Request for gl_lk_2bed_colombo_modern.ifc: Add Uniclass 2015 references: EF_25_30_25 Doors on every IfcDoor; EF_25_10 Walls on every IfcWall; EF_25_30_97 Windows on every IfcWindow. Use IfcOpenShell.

First a look at what the model holds.

```python
import ifcopenshell

model = ifcopenshell.open("gl_lk_2bed_colombo_modern.ifc")
print(model.schema)
print("classifications:", [c.Name for c in model.by_type("IfcClassification")])
for ifc_class in ("IfcDoor", "IfcRoof", "IfcStair", "IfcWall", "IfcWindow"):
    print(ifc_class, len(model.by_type(ifc_class)))
```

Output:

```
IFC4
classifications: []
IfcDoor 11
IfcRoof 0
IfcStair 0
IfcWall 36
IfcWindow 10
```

```python
import ifcopenshell
import ifcopenshell.api.classification

model = ifcopenshell.open("gl_lk_2bed_colombo_modern.ifc")

system = ifcopenshell.api.classification.add_classification(model, classification="Uniclass 2015")

codes = {
    "IfcDoor": ("EF_25_30_25", "Doors"),
    "IfcWall": ("EF_25_10", "Walls"),
    "IfcWindow": ("EF_25_30_97", "Windows"),
}
for ifc_class, (code, name) in codes.items():
    products = model.by_type(ifc_class)
    ifcopenshell.api.classification.add_reference(
        model, products=products, classification=system, identification=code, name=name
    )
    print(code, len(products))

model.write("gl_lk_2bed_colombo_modern_updated.ifc")
```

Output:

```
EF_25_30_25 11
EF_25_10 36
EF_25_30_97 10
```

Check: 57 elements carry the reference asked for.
